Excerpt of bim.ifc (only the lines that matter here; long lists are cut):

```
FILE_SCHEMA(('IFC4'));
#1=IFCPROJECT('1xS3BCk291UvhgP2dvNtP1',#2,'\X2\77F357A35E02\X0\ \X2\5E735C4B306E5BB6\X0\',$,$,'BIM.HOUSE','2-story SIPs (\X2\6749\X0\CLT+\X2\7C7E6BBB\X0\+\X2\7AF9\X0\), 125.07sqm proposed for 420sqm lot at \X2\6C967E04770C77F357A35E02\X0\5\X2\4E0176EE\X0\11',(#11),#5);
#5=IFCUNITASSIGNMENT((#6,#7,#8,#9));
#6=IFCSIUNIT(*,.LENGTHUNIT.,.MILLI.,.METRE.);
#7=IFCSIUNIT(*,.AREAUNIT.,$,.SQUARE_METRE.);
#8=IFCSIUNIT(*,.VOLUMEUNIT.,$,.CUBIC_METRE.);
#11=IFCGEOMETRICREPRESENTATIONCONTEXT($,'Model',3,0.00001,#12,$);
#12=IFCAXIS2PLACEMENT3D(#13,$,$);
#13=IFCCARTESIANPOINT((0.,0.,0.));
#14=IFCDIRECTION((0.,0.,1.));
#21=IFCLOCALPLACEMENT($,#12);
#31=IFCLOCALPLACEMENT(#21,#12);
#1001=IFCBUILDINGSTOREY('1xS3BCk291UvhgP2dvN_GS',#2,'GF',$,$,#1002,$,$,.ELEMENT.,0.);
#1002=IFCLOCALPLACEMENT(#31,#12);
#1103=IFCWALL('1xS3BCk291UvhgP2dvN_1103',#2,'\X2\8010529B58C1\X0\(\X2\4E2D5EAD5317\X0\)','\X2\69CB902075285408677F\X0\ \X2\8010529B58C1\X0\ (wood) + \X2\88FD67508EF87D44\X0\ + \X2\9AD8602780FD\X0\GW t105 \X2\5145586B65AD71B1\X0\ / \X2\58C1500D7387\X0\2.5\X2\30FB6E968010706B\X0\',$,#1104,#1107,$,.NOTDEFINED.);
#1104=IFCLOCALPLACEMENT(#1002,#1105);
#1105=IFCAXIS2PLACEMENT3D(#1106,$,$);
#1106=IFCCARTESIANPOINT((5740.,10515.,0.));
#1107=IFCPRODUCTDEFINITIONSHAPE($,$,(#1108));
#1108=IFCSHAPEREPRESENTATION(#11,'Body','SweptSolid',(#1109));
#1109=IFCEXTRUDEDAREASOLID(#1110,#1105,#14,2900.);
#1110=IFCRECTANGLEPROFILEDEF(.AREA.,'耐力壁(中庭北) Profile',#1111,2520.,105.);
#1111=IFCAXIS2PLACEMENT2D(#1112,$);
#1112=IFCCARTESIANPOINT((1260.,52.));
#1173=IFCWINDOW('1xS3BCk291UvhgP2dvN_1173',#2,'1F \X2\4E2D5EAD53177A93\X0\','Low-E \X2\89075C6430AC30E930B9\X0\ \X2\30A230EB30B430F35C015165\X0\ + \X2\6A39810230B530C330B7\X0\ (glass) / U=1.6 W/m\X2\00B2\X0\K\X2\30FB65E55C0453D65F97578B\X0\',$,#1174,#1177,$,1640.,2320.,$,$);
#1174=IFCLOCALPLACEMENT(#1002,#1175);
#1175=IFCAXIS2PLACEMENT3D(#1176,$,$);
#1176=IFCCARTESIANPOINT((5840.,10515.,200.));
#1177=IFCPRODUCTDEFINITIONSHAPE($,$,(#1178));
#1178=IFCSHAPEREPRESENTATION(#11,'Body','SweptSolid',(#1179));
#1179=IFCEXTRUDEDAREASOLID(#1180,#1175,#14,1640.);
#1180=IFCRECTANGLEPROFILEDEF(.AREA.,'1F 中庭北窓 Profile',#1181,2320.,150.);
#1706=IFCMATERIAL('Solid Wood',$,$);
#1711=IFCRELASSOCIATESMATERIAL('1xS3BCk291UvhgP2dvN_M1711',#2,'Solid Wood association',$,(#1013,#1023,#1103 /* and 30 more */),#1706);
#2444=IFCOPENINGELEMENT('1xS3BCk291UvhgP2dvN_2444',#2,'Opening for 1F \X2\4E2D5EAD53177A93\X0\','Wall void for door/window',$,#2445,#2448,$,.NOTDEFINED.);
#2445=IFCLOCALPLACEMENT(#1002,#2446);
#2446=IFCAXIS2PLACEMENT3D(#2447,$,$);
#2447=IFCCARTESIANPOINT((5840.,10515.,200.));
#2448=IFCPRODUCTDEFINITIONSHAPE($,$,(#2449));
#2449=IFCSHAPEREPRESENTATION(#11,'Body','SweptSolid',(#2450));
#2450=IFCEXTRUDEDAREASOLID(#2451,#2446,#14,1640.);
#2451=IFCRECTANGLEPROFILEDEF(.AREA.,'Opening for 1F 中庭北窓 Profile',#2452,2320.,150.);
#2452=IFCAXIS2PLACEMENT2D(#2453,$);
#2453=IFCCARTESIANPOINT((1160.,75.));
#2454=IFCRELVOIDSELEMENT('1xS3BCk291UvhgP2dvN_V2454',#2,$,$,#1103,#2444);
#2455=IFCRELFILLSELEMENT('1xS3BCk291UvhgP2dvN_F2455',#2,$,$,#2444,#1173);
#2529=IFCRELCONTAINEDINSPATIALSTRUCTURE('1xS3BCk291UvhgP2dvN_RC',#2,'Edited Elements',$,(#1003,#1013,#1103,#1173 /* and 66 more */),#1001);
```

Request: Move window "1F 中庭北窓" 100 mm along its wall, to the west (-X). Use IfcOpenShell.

```python
import ifcopenshell
import ifcopenshell.api.geometry
import ifcopenshell.util.placement

model = ifcopenshell.open("bim.ifc")

window = model.by_id(1173)
opening = window.FillsVoids[0].RelatingOpeningElement
wall = opening.VoidsElements[0].RelatingBuildingElement

wall_matrix = ifcopenshell.util.placement.get_local_placement(wall.ObjectPlacement)
shift = wall_matrix[:3, 0] * -100.0
before = ifcopenshell.util.placement.get_local_placement(window.ObjectPlacement)[:3, 3].copy()

# The window is not placed relative to its opening, so move both.
for product in (opening, window):
    matrix = ifcopenshell.util.placement.get_local_placement(product.ObjectPlacement)
    matrix[:3, 3] += shift
    ifcopenshell.api.geometry.edit_object_placement(model, product=product, matrix=matrix, is_si=False)

after = ifcopenshell.util.placement.get_local_placement(window.ObjectPlacement)[:3, 3]
print("window moved by", (after - before).round(3) + 0.0)

model.write("bim_rev.ifc")
```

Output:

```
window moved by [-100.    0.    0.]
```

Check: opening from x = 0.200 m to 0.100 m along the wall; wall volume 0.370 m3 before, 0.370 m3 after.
